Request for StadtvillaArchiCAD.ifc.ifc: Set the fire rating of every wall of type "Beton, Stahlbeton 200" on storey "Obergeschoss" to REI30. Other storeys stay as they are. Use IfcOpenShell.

First a look at what the model holds.

```python
import ifcopenshell
import ifcopenshell.util.element

model = ifcopenshell.open("StadtvillaArchiCAD.ifc.ifc")
print(model.schema)
storey = next(s for s in model.by_type("IfcBuildingStorey") if s.Name == "Obergeschoss")
walls = [e for e in ifcopenshell.util.element.get_decomposition(storey) if e.is_a("IfcWall")]
seen = {}
for e in walls:
    element_type = ifcopenshell.util.element.get_type(e)
    key = (element_type.Name if element_type != e and element_type else None, ifcopenshell.util.element.get_pset(e, "Pset_WallCommon", "FireRating"))
    seen[key] = seen.get(key, 0) + 1
for (name, value), count in sorted(seen.items(), key=str):
    print(count, "x", name, "|", value)
```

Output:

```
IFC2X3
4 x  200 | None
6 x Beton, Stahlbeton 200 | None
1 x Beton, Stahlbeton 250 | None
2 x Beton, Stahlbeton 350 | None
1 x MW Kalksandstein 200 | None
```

```python
import ifcopenshell
import ifcopenshell.api.pset
import ifcopenshell.util.element

model = ifcopenshell.open("StadtvillaArchiCAD.ifc.ifc")

storey = next(s for s in model.by_type("IfcBuildingStorey") if s.Name == "Obergeschoss")
walls = [e for e in ifcopenshell.util.element.get_decomposition(storey) if e.is_a("IfcWall")]

count = 0
for e in walls:
    element_type = ifcopenshell.util.element.get_type(e)
    if element_type in (None, e) or element_type.Name != "Beton, Stahlbeton 200":
        continue
    # add_pset returns the element's existing set when there is one.
    pset = ifcopenshell.api.pset.add_pset(model, product=e, name="Pset_WallCommon")
    ifcopenshell.api.pset.edit_pset(model, pset=pset, properties={"FireRating": "REI30"})
    count += 1

print(count, "walls updated")

model.write("StadtvillaArchiCAD.ifc_rev.ifc")
```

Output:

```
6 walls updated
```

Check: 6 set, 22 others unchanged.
